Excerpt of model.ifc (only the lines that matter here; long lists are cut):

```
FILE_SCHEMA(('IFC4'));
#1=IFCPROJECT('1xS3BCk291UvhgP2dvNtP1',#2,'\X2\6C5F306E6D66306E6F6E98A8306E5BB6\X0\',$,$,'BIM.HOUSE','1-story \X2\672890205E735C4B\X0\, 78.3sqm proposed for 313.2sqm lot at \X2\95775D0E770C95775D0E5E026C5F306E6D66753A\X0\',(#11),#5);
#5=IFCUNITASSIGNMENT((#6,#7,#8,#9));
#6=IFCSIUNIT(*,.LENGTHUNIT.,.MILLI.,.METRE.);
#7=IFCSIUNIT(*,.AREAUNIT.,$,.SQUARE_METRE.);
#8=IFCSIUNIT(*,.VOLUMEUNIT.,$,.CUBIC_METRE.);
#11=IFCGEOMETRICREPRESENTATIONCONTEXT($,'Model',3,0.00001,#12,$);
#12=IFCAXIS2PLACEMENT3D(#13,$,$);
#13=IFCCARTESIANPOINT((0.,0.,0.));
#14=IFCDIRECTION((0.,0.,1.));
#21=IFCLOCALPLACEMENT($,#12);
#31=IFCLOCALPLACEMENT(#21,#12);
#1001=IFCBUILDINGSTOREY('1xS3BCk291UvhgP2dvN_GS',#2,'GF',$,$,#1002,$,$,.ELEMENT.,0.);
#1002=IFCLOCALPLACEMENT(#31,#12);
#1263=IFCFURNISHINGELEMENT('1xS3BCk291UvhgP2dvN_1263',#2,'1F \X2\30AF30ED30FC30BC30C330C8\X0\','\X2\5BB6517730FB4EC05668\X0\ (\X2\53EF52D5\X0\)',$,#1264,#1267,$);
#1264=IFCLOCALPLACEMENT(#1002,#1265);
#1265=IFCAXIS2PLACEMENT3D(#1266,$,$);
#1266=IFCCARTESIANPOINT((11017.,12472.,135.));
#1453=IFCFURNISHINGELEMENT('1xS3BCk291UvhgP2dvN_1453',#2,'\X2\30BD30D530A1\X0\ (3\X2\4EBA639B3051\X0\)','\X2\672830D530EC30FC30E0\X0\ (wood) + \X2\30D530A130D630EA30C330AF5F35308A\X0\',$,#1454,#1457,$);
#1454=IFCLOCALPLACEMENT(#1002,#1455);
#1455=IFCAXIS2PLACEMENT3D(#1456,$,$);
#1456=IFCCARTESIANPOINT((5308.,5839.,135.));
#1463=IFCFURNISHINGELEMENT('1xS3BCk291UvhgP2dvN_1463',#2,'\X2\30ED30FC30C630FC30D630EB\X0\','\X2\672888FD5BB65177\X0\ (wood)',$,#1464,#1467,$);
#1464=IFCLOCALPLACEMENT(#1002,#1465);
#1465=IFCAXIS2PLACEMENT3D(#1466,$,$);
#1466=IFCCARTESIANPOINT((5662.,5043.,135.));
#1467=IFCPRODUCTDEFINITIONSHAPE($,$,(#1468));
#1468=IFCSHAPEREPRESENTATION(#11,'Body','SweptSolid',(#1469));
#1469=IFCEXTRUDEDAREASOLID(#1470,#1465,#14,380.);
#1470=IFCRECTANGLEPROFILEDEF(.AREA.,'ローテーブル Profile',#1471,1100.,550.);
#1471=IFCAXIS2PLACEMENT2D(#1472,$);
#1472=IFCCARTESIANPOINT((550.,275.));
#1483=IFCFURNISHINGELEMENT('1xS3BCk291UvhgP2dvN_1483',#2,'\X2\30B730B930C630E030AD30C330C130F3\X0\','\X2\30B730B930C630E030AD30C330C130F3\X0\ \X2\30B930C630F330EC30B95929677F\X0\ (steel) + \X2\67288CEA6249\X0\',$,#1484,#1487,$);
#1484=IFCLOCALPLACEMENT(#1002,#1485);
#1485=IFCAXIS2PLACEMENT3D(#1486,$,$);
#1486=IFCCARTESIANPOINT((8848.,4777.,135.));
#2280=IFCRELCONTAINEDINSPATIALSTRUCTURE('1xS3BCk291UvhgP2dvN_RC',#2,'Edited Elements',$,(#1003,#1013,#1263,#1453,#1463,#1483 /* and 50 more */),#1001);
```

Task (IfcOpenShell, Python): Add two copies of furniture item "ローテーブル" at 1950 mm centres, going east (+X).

```python
import numpy as np
import ifcopenshell
import ifcopenshell.api.geometry
import ifcopenshell.api.root
import ifcopenshell.util.element
import ifcopenshell.util.placement
import ifcopenshell.util.unit

model = ifcopenshell.open("model.ifc")
unit_scale = ifcopenshell.util.unit.calculate_unit_scale(model)


def reuse_history(source, copy):
    """copy_class also copies each property set's owner history, people and application; keep the originals."""
    for rel in copy.IsDefinedBy:
        if rel.is_a("IfcRelDefinesByProperties") and (history := rel.RelatingPropertyDefinition.OwnerHistory):
            rel.RelatingPropertyDefinition.OwnerHistory = source.OwnerHistory
            ifcopenshell.util.element.remove_deep2(model, history)


source = model.by_id(1463)
base = ifcopenshell.util.placement.get_local_placement(source.ObjectPlacement)
step = np.array([1.0, 0.0, 0.0]) * 1.95 / unit_scale

for i in range(1, 3):
    copy = ifcopenshell.api.root.copy_class(model, product=source)
    copy.Representation = ifcopenshell.util.element.copy_deep(
        model, source.Representation, exclude=["IfcGeometricRepresentationContext", "IfcRepresentationMap"]
    )
    reuse_history(source, copy)
    matrix = base.copy()
    matrix[:3, 3] += i * step
    print("added at", matrix[:3, 3].round(3) + 0.0)
    ifcopenshell.api.geometry.edit_object_placement(model, product=copy, matrix=matrix, is_si=False)

model.write("model_v2.ifc")
```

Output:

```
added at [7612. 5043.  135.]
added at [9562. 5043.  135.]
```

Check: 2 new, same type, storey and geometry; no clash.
